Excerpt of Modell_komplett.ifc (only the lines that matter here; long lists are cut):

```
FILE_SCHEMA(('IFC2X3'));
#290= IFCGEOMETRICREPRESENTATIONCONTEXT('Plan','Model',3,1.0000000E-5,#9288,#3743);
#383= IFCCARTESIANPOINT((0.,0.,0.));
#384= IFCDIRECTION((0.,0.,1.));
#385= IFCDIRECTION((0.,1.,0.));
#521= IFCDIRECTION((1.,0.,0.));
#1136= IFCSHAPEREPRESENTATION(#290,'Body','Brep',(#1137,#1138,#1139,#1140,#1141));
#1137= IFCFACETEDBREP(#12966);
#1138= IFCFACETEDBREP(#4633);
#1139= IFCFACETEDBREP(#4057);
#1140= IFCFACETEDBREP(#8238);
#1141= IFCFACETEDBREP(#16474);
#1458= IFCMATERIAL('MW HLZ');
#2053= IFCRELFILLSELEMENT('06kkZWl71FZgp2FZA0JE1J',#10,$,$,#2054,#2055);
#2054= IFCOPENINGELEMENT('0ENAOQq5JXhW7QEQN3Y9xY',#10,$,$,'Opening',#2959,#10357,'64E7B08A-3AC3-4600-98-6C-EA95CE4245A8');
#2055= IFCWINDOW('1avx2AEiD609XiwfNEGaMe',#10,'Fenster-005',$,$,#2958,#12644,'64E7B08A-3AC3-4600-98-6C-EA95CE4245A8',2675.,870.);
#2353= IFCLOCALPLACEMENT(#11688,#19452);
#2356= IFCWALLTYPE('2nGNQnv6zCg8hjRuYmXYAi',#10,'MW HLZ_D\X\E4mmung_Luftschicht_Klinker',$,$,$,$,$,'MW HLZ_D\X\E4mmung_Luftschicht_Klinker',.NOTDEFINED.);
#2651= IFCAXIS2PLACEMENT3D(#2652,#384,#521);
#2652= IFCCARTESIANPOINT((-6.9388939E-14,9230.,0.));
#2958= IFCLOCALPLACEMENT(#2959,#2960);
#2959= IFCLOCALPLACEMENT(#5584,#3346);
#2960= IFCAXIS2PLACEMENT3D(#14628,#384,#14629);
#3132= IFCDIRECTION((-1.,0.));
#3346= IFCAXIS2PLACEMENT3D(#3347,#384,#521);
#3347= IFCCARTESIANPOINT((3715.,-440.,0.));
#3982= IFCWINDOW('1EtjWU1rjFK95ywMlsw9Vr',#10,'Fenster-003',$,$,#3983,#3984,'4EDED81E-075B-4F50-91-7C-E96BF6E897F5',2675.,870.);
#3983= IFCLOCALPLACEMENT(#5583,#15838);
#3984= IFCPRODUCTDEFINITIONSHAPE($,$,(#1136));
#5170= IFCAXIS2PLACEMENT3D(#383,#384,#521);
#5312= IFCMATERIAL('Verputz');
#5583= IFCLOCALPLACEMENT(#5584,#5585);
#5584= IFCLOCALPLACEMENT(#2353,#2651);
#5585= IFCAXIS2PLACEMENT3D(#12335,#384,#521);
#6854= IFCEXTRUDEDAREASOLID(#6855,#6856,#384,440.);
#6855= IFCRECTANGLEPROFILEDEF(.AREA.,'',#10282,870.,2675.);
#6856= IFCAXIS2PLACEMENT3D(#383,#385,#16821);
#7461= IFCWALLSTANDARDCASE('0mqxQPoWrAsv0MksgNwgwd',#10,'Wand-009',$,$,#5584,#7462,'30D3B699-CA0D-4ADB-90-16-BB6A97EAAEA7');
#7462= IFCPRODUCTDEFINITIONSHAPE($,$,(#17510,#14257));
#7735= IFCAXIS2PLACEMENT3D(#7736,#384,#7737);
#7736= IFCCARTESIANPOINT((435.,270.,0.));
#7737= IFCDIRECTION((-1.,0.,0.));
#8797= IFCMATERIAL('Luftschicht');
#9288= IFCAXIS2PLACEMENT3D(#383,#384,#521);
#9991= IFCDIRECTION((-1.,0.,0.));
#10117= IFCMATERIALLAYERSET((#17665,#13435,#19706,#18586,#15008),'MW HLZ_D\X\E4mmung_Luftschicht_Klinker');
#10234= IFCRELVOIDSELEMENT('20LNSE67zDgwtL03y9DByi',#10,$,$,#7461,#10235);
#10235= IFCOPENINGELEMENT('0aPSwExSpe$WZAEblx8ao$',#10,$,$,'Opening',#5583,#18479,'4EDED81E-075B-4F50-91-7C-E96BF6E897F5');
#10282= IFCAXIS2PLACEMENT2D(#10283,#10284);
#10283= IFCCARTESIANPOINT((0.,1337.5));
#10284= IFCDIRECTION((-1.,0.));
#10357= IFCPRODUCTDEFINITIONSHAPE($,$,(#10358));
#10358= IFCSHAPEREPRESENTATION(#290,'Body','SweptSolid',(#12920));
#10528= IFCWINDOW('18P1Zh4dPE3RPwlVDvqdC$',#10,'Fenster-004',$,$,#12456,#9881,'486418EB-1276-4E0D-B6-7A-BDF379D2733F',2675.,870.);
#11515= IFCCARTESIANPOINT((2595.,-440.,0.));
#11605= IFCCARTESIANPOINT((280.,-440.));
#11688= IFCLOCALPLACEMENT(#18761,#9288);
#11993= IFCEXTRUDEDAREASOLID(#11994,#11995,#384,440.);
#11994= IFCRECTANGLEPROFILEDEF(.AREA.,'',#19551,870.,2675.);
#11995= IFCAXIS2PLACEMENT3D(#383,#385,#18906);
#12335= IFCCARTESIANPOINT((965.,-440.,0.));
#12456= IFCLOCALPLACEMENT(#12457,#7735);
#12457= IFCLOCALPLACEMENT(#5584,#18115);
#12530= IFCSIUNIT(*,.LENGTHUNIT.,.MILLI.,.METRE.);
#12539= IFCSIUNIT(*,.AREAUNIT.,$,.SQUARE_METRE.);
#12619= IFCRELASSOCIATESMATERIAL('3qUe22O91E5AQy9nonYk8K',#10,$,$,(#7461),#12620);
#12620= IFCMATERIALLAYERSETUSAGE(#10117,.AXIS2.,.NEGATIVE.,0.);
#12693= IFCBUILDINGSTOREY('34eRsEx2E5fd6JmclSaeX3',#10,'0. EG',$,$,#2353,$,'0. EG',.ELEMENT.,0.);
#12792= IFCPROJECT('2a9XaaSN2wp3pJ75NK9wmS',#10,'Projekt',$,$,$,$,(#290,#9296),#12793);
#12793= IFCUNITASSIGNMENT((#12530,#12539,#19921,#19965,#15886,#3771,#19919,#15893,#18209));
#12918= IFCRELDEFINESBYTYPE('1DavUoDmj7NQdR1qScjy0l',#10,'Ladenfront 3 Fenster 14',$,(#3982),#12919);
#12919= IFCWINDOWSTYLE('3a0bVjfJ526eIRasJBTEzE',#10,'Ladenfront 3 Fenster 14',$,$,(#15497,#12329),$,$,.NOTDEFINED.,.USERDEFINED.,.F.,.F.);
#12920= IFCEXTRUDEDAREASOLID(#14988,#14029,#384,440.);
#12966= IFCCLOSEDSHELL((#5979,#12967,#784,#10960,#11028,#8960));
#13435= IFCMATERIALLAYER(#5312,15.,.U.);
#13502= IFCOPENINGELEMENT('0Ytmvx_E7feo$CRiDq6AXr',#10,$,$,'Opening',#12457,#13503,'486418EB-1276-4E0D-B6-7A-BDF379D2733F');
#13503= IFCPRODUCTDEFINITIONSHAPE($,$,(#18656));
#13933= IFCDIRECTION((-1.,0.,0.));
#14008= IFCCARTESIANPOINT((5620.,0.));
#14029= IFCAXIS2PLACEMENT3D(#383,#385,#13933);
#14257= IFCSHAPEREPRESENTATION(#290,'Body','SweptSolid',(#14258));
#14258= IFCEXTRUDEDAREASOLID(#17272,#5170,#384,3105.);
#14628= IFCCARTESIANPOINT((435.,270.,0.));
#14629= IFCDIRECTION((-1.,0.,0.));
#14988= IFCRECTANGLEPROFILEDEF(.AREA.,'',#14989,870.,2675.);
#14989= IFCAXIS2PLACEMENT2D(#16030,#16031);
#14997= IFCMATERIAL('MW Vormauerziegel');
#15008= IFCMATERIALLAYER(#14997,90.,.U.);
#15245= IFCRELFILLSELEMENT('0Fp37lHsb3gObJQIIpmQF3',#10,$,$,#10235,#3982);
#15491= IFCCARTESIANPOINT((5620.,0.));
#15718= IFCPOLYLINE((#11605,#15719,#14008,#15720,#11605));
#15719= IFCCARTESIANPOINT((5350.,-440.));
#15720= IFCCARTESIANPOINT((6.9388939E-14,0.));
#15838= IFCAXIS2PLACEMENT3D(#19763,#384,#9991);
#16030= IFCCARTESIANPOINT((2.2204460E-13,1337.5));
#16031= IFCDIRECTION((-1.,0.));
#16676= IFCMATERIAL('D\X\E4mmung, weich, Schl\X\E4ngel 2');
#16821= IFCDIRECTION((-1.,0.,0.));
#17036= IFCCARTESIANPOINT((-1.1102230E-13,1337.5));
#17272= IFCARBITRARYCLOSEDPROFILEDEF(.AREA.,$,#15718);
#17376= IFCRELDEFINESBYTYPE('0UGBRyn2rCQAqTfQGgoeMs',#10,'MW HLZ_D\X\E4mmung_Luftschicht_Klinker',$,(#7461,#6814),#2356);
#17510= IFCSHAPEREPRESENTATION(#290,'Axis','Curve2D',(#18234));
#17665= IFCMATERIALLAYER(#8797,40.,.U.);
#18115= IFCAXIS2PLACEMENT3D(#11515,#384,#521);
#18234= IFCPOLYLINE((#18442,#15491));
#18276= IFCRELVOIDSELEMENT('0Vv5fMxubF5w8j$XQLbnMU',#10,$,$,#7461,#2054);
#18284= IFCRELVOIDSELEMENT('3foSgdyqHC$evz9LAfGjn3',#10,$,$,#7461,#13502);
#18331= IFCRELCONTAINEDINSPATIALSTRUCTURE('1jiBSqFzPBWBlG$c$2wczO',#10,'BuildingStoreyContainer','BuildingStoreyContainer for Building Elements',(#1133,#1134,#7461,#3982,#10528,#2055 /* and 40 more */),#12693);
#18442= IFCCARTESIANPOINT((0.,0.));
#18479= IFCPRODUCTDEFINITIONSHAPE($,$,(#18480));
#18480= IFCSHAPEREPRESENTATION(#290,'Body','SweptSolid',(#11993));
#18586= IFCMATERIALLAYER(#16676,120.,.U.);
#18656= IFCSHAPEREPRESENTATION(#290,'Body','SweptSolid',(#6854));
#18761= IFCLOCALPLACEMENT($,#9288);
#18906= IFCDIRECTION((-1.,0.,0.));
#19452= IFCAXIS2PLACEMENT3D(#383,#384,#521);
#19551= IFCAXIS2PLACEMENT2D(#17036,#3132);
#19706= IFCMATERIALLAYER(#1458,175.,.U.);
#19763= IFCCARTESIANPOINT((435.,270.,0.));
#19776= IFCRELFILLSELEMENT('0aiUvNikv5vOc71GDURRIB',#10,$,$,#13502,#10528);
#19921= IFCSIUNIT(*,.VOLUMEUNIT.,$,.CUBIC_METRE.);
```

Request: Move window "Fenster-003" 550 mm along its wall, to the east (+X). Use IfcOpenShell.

```python
import ifcopenshell
import ifcopenshell.api.geometry
import ifcopenshell.util.placement

model = ifcopenshell.open("Modell_komplett.ifc")

window = model.by_guid("1EtjWU1rjFK95ywMlsw9Vr")
opening = window.FillsVoids[0].RelatingOpeningElement
wall = opening.VoidsElements[0].RelatingBuildingElement

wall_matrix = ifcopenshell.util.placement.get_local_placement(wall.ObjectPlacement)
shift = wall_matrix[:3, 0] * 550.0
before = ifcopenshell.util.placement.get_local_placement(window.ObjectPlacement)[:3, 3].copy()

# The window is placed relative to its opening, so it follows when the opening moves.
matrix = ifcopenshell.util.placement.get_local_placement(opening.ObjectPlacement)
matrix[:3, 3] += shift
ifcopenshell.api.geometry.edit_object_placement(
    model, product=opening, matrix=matrix, is_si=False, should_transform_children=True
)

after = ifcopenshell.util.placement.get_local_placement(window.ObjectPlacement)[:3, 3]
print("window moved by", (after - before).round(3) + 0.0)

model.write("Modell_komplett-out.ifc")
```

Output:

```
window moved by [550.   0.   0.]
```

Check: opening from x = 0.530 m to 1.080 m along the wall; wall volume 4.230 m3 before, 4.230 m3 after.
